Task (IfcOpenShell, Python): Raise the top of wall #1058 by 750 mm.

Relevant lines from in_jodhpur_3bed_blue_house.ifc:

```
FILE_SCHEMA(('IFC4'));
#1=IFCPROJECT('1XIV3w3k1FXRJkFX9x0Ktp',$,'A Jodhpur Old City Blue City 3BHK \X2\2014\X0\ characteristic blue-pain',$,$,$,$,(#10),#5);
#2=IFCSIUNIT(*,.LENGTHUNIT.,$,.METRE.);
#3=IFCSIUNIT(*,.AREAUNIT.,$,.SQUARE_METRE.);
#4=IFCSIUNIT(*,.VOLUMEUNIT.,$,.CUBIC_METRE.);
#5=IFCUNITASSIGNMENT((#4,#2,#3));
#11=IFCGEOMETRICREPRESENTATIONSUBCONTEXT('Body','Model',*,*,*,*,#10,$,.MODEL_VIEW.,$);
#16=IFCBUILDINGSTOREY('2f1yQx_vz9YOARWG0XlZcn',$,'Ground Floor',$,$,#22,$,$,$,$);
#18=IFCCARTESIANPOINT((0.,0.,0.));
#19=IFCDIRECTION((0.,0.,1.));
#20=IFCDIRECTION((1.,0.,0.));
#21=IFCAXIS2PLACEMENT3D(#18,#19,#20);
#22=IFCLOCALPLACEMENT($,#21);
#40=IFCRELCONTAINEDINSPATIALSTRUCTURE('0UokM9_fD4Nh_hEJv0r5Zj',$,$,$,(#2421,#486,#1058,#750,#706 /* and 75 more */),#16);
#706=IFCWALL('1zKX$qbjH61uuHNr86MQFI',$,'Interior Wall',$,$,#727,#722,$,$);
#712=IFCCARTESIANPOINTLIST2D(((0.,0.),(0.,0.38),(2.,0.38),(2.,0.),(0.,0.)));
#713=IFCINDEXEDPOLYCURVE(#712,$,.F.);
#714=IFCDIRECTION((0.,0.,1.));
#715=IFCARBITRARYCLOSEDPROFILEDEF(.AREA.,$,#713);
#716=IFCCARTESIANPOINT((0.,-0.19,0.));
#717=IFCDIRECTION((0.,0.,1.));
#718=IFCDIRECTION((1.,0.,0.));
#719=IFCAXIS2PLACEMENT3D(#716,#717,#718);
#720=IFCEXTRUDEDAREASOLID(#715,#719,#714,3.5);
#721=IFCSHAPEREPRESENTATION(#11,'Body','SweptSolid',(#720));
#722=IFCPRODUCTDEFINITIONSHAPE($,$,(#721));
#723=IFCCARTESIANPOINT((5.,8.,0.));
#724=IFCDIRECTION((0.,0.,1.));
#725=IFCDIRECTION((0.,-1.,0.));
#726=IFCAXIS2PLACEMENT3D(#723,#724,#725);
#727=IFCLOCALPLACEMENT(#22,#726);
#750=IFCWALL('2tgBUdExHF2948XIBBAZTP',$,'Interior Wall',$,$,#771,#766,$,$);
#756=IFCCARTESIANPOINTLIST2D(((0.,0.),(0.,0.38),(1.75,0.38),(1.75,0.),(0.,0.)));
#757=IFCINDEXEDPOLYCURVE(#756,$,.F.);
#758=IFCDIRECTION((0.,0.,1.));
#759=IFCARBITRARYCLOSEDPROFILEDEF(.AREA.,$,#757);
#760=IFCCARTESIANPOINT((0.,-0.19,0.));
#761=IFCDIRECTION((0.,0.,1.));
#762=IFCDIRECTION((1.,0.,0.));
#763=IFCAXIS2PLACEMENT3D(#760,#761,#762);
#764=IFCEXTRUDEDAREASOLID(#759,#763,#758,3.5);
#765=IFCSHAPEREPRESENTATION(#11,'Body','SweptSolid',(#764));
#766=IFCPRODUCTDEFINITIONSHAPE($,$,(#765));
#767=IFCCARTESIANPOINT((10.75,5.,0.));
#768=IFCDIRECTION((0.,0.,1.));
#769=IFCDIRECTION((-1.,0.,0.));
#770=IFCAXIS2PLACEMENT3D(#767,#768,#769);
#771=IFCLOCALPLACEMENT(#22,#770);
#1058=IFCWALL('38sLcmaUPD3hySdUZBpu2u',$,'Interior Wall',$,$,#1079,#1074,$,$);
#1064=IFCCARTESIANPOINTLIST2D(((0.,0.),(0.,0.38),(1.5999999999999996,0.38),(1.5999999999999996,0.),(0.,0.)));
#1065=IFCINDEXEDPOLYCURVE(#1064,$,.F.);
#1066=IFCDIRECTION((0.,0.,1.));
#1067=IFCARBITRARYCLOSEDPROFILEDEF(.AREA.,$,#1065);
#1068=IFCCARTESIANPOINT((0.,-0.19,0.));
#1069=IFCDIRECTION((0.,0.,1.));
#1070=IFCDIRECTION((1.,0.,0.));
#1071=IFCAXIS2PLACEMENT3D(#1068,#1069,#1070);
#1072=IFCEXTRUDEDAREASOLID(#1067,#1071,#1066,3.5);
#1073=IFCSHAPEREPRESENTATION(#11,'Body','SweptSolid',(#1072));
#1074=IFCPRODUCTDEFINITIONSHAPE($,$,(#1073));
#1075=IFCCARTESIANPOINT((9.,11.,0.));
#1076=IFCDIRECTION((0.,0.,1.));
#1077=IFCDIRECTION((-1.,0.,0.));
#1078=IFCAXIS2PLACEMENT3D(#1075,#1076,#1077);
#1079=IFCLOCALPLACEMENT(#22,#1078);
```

```python
import ifcopenshell
import ifcopenshell.geom
import ifcopenshell.util.representation
import ifcopenshell.util.shape
import ifcopenshell.util.unit

model = ifcopenshell.open("in_jodhpur_3bed_blue_house.ifc")
unit_scale = ifcopenshell.util.unit.calculate_unit_scale(model)
settings = ifcopenshell.geom.settings()


def volume(element):
    """Net volume in cubic metres, openings subtracted."""
    shape = ifcopenshell.geom.create_shape(settings, element)
    return ifcopenshell.util.shape.get_volume(shape.geometry)


wall = model.by_guid("38sLcmaUPD3hySdUZBpu2u")
before = volume(wall)

body = ifcopenshell.util.representation.get_representation(wall, "Model", "Body")
solid = body.Items[0]
old_height = solid.Depth
solid.Depth += 0.75 / unit_scale
after = volume(wall)

print(f"height {old_height:g} -> {solid.Depth:g}, volume {before:.3f} -> {after:.3f} m3")

model.write("in_jodhpur_3bed_blue_house_v2.ifc")
```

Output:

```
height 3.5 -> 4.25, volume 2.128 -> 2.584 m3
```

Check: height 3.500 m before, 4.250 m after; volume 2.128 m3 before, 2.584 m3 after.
